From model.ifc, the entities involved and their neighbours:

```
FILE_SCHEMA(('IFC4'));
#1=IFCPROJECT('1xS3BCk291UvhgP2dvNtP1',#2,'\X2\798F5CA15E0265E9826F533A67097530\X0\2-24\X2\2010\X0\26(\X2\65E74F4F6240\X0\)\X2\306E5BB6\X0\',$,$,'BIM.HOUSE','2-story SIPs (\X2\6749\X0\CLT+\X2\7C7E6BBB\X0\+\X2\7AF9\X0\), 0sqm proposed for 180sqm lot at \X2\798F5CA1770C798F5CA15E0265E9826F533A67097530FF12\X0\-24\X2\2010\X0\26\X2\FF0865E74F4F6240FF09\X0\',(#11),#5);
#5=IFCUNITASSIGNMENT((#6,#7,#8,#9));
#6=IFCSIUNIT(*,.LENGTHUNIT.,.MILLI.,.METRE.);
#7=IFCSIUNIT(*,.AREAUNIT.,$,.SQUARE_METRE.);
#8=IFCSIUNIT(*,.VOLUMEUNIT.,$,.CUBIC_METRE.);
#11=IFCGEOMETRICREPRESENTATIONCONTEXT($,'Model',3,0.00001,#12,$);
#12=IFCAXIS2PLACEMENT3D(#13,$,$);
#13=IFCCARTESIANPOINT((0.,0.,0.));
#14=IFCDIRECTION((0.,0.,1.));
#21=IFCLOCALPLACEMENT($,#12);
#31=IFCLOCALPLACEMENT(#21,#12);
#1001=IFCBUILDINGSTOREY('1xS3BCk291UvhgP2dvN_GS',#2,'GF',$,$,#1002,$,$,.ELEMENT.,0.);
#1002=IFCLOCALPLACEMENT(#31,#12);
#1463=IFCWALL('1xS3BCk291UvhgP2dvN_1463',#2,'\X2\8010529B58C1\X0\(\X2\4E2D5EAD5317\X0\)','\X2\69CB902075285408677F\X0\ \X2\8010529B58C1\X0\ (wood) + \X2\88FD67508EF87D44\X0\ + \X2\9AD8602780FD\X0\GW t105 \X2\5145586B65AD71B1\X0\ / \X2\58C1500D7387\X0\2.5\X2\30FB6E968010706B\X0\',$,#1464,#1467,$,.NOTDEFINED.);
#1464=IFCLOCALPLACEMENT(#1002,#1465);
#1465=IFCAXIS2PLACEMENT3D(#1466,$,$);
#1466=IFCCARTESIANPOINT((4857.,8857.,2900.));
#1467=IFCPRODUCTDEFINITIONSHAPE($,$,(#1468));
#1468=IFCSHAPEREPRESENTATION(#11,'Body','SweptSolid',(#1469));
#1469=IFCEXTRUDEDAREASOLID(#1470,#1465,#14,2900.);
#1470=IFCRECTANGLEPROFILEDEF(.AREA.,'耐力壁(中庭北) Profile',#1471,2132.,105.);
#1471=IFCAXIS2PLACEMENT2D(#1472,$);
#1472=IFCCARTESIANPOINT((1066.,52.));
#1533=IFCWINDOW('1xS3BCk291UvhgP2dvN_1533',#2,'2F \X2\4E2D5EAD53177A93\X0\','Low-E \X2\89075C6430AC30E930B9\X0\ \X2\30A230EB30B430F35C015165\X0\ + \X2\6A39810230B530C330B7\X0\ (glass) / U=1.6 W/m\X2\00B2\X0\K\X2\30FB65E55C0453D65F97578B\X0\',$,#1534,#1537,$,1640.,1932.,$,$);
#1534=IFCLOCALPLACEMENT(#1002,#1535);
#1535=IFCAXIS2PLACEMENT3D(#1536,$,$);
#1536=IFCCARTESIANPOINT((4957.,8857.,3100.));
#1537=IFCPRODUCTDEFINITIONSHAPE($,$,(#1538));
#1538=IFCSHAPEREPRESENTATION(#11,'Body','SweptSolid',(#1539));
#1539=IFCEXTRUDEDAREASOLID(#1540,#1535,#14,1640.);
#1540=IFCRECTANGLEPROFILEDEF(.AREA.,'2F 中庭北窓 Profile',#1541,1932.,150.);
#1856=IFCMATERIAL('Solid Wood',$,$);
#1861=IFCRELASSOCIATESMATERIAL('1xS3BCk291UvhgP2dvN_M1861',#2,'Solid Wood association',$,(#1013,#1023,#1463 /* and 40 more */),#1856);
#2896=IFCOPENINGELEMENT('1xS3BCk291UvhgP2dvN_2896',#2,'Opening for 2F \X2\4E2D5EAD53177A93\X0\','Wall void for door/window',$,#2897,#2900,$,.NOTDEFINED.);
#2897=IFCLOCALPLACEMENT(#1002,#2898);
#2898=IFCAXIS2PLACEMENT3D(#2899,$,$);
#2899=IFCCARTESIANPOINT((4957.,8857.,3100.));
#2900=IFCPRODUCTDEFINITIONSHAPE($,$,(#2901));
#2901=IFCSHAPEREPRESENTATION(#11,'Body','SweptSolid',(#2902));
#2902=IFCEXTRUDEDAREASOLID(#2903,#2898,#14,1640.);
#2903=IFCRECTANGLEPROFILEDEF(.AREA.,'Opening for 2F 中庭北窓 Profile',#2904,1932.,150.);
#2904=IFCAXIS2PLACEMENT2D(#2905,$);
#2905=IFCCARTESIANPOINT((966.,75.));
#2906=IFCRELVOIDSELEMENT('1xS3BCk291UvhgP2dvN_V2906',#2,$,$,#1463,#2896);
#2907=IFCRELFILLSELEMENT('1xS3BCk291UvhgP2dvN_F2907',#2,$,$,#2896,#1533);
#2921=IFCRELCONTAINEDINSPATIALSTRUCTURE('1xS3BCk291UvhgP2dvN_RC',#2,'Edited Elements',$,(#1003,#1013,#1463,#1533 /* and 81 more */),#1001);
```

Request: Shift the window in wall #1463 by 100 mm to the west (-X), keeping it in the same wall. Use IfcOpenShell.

```python
import ifcopenshell
import ifcopenshell.api.geometry
import ifcopenshell.util.placement

model = ifcopenshell.open("model.ifc")

window = model.by_guid("1xS3BCk291UvhgP2dvN_1533")
opening = window.FillsVoids[0].RelatingOpeningElement
wall = opening.VoidsElements[0].RelatingBuildingElement

wall_matrix = ifcopenshell.util.placement.get_local_placement(wall.ObjectPlacement)
shift = wall_matrix[:3, 0] * -100.0
before = ifcopenshell.util.placement.get_local_placement(window.ObjectPlacement)[:3, 3].copy()

# The window is not placed relative to its opening, so move both.
for product in (opening, window):
    matrix = ifcopenshell.util.placement.get_local_placement(product.ObjectPlacement)
    matrix[:3, 3] += shift
    ifcopenshell.api.geometry.edit_object_placement(model, product=product, matrix=matrix, is_si=False)

after = ifcopenshell.util.placement.get_local_placement(window.ObjectPlacement)[:3, 3]
print("window moved by", (after - before).round(3) + 0.0)

model.write("model-out.ifc")
```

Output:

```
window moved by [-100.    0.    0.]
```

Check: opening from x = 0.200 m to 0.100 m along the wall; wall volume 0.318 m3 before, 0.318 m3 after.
